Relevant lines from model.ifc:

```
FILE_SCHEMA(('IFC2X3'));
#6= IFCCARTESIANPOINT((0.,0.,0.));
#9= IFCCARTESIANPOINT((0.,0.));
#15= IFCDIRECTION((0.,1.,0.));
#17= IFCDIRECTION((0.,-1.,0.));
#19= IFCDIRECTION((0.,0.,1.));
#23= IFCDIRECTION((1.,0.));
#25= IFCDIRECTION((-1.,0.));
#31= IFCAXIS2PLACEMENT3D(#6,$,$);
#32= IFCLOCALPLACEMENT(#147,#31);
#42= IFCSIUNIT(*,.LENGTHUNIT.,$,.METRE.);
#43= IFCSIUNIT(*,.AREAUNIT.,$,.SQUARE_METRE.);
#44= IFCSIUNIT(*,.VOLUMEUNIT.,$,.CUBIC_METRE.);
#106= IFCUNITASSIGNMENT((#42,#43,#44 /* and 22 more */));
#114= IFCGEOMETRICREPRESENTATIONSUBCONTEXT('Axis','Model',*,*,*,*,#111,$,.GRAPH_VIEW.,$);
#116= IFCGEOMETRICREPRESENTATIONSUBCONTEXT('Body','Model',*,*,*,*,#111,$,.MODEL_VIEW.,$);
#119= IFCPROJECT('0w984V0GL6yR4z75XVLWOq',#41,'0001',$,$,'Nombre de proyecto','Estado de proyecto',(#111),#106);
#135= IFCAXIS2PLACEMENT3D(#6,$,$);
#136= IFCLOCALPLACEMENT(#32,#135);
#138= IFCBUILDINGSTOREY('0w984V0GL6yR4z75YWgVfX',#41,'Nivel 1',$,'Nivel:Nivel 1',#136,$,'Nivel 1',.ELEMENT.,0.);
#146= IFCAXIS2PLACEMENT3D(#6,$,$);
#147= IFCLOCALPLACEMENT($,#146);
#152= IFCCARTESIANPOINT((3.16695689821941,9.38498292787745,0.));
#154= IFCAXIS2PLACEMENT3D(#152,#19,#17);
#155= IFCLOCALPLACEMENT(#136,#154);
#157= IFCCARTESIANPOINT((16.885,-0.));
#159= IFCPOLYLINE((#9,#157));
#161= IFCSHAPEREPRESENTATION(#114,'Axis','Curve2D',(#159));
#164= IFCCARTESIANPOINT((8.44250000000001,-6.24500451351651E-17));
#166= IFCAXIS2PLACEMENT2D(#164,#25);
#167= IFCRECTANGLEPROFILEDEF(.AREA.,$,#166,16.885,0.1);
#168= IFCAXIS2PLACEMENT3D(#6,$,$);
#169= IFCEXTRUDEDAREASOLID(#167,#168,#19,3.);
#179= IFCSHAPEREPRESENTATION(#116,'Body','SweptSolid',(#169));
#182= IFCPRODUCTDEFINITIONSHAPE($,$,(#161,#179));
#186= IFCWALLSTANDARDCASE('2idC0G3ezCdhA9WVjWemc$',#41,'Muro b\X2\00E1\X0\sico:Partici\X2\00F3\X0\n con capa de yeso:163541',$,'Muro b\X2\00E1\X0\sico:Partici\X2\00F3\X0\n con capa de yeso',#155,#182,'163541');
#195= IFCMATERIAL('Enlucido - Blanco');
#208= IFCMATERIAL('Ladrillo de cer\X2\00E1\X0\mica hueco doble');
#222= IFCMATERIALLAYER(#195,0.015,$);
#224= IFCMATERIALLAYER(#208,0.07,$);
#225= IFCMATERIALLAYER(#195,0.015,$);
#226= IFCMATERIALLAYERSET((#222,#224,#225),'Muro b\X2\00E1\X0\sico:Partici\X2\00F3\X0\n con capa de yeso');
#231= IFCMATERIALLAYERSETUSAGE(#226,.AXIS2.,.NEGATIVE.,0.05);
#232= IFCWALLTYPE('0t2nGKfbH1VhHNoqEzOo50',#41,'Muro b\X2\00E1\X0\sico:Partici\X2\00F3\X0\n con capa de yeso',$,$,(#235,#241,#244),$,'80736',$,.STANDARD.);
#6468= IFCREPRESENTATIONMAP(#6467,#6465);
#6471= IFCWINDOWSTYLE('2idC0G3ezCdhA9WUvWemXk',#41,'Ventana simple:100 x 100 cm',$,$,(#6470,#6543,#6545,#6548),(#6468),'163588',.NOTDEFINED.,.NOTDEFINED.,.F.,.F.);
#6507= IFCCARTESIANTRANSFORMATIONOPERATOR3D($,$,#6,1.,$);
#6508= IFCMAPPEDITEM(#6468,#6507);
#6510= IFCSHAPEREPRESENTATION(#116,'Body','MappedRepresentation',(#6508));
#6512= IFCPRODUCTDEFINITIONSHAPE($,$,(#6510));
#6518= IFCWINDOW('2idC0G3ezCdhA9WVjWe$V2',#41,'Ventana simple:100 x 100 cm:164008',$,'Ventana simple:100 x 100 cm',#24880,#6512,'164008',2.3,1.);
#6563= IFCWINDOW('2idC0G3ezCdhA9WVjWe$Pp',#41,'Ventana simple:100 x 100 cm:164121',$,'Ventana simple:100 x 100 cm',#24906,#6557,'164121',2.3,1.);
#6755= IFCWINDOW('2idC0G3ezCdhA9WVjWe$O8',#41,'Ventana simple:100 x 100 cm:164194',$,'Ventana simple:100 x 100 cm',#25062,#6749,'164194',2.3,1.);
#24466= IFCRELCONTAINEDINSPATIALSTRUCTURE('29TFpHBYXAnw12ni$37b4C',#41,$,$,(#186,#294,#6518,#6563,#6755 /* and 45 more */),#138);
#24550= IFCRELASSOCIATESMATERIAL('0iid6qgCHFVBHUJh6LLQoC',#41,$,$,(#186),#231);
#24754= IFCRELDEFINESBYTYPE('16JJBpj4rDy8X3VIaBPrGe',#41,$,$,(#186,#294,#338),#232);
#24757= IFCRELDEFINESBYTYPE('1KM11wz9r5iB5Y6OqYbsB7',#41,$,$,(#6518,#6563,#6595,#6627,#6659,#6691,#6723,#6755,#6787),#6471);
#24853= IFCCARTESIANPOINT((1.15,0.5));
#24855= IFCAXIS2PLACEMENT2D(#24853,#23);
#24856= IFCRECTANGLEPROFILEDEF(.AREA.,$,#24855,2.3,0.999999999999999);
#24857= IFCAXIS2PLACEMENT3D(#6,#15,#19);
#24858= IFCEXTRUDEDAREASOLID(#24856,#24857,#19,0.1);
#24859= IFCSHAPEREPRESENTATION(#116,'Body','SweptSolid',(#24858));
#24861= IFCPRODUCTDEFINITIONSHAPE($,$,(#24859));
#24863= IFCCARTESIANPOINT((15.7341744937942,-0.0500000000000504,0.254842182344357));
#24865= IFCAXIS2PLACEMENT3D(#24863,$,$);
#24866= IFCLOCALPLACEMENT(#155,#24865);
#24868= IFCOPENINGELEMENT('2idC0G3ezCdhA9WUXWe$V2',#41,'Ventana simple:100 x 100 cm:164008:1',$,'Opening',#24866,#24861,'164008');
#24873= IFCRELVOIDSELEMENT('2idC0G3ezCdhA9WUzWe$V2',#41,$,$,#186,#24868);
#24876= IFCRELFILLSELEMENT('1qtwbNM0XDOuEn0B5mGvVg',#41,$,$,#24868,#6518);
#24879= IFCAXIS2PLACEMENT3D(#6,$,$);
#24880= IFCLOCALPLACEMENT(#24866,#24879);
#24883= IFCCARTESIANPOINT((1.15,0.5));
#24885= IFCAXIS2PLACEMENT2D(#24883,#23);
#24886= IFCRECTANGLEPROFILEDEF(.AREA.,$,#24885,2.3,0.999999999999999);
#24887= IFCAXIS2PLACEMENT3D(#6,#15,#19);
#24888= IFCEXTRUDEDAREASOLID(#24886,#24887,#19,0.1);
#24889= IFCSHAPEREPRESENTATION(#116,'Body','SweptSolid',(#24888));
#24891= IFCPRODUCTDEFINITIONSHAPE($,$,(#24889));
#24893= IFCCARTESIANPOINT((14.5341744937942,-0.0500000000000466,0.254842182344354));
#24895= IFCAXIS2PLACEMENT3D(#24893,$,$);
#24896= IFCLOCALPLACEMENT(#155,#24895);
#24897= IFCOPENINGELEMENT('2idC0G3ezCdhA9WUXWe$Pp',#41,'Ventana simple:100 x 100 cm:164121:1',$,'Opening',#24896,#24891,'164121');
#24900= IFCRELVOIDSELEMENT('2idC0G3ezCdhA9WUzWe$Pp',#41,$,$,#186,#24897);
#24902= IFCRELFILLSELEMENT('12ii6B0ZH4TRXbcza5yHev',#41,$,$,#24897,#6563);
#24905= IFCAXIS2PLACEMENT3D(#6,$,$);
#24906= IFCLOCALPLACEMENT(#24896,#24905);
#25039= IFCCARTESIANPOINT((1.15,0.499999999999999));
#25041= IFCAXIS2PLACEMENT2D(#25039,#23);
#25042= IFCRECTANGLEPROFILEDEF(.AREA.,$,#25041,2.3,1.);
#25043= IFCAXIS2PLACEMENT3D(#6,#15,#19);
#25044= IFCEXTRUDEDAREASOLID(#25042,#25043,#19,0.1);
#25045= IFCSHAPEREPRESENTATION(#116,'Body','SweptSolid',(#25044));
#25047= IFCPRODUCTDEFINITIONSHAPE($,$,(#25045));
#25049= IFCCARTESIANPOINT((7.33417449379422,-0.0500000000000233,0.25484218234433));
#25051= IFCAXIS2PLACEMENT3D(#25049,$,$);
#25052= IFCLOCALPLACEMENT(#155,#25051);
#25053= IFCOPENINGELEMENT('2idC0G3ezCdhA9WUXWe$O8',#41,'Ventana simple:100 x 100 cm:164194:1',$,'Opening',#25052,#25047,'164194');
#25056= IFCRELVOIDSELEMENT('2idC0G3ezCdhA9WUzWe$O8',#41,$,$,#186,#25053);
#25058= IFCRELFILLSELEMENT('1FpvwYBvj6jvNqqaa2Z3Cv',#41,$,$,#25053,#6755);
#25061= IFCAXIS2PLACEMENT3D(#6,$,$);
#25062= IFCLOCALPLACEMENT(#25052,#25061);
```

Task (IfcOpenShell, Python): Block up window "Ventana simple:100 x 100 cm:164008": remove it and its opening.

```python
import ifcopenshell
import ifcopenshell.api.feature
import ifcopenshell.api.root
import ifcopenshell.geom
import ifcopenshell.util.shape

model = ifcopenshell.open("model.ifc")
settings = ifcopenshell.geom.settings()


def volume(element):
    """Net volume in cubic metres, openings subtracted."""
    shape = ifcopenshell.geom.create_shape(settings, element)
    return ifcopenshell.util.shape.get_volume(shape.geometry)


window = model.by_guid("2idC0G3ezCdhA9WVjWe$V2")
opening = window.FillsVoids[0].RelatingOpeningElement
wall = opening.VoidsElements[0].RelatingBuildingElement
before = volume(wall)

ifcopenshell.api.root.remove_product(model, product=window)
ifcopenshell.api.feature.remove_feature(model, feature=opening)

after = volume(wall)

print(f"wall volume {before:.3f} -> {after:.3f} m3")

model.write("model_edited.ifc")
```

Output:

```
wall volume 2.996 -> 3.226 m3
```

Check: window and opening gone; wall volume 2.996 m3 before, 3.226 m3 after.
